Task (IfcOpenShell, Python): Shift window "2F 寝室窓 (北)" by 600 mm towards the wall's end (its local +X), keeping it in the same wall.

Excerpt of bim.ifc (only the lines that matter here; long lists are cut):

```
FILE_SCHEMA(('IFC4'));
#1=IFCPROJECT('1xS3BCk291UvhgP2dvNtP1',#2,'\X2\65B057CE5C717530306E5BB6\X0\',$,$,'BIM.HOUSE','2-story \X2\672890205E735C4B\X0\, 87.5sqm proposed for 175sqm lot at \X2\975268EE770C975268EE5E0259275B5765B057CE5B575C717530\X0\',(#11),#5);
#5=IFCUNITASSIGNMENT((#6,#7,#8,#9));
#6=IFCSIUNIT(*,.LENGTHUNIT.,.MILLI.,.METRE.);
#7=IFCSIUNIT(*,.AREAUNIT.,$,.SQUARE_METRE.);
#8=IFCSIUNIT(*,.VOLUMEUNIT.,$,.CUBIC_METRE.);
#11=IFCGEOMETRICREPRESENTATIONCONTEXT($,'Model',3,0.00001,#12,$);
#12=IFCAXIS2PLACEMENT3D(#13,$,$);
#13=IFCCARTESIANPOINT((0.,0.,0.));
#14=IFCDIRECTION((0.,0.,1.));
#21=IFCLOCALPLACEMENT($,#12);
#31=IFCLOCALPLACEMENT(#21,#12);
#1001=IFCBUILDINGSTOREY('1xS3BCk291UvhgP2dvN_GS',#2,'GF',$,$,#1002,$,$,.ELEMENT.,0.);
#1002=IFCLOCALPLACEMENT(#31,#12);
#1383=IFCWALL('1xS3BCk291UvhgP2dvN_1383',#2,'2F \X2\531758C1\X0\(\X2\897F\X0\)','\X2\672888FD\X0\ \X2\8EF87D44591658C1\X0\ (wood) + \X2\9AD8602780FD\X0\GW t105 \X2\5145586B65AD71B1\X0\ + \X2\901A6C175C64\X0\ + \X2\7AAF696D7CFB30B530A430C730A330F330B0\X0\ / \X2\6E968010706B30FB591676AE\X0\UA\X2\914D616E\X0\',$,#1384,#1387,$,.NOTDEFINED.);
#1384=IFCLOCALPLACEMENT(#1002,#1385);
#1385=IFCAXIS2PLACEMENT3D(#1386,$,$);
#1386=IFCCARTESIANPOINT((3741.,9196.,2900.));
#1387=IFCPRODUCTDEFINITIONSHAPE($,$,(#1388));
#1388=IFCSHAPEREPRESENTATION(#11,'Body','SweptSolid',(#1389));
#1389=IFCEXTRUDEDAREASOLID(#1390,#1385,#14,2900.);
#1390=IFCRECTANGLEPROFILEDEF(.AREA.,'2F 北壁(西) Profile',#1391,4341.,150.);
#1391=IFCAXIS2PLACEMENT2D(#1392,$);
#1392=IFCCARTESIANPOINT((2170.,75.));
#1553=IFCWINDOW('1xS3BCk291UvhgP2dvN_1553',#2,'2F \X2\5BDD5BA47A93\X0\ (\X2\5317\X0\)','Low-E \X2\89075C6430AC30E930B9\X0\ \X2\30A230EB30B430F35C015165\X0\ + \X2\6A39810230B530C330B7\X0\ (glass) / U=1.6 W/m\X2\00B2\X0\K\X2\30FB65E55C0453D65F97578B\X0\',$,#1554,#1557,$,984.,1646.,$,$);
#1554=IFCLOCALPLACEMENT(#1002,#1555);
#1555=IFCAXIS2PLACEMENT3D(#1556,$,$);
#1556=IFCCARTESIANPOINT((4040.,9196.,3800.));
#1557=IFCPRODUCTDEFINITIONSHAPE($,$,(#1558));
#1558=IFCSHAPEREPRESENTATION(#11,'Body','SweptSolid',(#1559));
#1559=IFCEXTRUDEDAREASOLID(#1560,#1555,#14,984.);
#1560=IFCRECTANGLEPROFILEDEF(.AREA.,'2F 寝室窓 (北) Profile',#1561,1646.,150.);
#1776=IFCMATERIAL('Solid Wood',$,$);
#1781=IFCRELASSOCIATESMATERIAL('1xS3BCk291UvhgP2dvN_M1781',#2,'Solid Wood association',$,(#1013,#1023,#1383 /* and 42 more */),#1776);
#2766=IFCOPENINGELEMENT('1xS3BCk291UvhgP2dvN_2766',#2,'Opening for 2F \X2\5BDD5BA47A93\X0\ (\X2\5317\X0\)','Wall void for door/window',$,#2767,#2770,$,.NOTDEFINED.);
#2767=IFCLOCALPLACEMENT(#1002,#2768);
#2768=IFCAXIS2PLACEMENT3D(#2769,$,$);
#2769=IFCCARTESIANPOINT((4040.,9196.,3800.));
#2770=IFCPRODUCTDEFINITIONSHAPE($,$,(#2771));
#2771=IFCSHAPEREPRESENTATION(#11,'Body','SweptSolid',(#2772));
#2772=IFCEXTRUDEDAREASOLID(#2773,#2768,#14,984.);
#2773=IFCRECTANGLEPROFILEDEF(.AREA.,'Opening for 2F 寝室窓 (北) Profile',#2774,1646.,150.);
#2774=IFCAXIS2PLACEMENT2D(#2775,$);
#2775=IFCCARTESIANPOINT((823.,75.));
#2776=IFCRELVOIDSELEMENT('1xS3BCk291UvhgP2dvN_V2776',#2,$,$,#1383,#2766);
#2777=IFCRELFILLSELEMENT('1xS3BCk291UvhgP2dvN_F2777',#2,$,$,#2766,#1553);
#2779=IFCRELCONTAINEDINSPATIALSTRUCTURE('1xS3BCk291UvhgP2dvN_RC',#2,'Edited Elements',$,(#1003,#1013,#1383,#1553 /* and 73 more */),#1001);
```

```python
import ifcopenshell
import ifcopenshell.api.geometry
import ifcopenshell.util.placement

model = ifcopenshell.open("bim.ifc")

window = model.by_id(1553)
opening = window.FillsVoids[0].RelatingOpeningElement
wall = opening.VoidsElements[0].RelatingBuildingElement

wall_matrix = ifcopenshell.util.placement.get_local_placement(wall.ObjectPlacement)
shift = wall_matrix[:3, 0] * 600.0
before = ifcopenshell.util.placement.get_local_placement(window.ObjectPlacement)[:3, 3].copy()

# The window is not placed relative to its opening, so move both.
for product in (opening, window):
    matrix = ifcopenshell.util.placement.get_local_placement(product.ObjectPlacement)
    matrix[:3, 3] += shift
    ifcopenshell.api.geometry.edit_object_placement(model, product=product, matrix=matrix, is_si=False)

after = ifcopenshell.util.placement.get_local_placement(window.ObjectPlacement)[:3, 3]
print("window moved by", (after - before).round(3) + 0.0)

model.write("bim-out.ifc")
```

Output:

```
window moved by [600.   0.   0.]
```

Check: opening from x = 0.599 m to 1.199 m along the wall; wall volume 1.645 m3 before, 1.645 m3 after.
